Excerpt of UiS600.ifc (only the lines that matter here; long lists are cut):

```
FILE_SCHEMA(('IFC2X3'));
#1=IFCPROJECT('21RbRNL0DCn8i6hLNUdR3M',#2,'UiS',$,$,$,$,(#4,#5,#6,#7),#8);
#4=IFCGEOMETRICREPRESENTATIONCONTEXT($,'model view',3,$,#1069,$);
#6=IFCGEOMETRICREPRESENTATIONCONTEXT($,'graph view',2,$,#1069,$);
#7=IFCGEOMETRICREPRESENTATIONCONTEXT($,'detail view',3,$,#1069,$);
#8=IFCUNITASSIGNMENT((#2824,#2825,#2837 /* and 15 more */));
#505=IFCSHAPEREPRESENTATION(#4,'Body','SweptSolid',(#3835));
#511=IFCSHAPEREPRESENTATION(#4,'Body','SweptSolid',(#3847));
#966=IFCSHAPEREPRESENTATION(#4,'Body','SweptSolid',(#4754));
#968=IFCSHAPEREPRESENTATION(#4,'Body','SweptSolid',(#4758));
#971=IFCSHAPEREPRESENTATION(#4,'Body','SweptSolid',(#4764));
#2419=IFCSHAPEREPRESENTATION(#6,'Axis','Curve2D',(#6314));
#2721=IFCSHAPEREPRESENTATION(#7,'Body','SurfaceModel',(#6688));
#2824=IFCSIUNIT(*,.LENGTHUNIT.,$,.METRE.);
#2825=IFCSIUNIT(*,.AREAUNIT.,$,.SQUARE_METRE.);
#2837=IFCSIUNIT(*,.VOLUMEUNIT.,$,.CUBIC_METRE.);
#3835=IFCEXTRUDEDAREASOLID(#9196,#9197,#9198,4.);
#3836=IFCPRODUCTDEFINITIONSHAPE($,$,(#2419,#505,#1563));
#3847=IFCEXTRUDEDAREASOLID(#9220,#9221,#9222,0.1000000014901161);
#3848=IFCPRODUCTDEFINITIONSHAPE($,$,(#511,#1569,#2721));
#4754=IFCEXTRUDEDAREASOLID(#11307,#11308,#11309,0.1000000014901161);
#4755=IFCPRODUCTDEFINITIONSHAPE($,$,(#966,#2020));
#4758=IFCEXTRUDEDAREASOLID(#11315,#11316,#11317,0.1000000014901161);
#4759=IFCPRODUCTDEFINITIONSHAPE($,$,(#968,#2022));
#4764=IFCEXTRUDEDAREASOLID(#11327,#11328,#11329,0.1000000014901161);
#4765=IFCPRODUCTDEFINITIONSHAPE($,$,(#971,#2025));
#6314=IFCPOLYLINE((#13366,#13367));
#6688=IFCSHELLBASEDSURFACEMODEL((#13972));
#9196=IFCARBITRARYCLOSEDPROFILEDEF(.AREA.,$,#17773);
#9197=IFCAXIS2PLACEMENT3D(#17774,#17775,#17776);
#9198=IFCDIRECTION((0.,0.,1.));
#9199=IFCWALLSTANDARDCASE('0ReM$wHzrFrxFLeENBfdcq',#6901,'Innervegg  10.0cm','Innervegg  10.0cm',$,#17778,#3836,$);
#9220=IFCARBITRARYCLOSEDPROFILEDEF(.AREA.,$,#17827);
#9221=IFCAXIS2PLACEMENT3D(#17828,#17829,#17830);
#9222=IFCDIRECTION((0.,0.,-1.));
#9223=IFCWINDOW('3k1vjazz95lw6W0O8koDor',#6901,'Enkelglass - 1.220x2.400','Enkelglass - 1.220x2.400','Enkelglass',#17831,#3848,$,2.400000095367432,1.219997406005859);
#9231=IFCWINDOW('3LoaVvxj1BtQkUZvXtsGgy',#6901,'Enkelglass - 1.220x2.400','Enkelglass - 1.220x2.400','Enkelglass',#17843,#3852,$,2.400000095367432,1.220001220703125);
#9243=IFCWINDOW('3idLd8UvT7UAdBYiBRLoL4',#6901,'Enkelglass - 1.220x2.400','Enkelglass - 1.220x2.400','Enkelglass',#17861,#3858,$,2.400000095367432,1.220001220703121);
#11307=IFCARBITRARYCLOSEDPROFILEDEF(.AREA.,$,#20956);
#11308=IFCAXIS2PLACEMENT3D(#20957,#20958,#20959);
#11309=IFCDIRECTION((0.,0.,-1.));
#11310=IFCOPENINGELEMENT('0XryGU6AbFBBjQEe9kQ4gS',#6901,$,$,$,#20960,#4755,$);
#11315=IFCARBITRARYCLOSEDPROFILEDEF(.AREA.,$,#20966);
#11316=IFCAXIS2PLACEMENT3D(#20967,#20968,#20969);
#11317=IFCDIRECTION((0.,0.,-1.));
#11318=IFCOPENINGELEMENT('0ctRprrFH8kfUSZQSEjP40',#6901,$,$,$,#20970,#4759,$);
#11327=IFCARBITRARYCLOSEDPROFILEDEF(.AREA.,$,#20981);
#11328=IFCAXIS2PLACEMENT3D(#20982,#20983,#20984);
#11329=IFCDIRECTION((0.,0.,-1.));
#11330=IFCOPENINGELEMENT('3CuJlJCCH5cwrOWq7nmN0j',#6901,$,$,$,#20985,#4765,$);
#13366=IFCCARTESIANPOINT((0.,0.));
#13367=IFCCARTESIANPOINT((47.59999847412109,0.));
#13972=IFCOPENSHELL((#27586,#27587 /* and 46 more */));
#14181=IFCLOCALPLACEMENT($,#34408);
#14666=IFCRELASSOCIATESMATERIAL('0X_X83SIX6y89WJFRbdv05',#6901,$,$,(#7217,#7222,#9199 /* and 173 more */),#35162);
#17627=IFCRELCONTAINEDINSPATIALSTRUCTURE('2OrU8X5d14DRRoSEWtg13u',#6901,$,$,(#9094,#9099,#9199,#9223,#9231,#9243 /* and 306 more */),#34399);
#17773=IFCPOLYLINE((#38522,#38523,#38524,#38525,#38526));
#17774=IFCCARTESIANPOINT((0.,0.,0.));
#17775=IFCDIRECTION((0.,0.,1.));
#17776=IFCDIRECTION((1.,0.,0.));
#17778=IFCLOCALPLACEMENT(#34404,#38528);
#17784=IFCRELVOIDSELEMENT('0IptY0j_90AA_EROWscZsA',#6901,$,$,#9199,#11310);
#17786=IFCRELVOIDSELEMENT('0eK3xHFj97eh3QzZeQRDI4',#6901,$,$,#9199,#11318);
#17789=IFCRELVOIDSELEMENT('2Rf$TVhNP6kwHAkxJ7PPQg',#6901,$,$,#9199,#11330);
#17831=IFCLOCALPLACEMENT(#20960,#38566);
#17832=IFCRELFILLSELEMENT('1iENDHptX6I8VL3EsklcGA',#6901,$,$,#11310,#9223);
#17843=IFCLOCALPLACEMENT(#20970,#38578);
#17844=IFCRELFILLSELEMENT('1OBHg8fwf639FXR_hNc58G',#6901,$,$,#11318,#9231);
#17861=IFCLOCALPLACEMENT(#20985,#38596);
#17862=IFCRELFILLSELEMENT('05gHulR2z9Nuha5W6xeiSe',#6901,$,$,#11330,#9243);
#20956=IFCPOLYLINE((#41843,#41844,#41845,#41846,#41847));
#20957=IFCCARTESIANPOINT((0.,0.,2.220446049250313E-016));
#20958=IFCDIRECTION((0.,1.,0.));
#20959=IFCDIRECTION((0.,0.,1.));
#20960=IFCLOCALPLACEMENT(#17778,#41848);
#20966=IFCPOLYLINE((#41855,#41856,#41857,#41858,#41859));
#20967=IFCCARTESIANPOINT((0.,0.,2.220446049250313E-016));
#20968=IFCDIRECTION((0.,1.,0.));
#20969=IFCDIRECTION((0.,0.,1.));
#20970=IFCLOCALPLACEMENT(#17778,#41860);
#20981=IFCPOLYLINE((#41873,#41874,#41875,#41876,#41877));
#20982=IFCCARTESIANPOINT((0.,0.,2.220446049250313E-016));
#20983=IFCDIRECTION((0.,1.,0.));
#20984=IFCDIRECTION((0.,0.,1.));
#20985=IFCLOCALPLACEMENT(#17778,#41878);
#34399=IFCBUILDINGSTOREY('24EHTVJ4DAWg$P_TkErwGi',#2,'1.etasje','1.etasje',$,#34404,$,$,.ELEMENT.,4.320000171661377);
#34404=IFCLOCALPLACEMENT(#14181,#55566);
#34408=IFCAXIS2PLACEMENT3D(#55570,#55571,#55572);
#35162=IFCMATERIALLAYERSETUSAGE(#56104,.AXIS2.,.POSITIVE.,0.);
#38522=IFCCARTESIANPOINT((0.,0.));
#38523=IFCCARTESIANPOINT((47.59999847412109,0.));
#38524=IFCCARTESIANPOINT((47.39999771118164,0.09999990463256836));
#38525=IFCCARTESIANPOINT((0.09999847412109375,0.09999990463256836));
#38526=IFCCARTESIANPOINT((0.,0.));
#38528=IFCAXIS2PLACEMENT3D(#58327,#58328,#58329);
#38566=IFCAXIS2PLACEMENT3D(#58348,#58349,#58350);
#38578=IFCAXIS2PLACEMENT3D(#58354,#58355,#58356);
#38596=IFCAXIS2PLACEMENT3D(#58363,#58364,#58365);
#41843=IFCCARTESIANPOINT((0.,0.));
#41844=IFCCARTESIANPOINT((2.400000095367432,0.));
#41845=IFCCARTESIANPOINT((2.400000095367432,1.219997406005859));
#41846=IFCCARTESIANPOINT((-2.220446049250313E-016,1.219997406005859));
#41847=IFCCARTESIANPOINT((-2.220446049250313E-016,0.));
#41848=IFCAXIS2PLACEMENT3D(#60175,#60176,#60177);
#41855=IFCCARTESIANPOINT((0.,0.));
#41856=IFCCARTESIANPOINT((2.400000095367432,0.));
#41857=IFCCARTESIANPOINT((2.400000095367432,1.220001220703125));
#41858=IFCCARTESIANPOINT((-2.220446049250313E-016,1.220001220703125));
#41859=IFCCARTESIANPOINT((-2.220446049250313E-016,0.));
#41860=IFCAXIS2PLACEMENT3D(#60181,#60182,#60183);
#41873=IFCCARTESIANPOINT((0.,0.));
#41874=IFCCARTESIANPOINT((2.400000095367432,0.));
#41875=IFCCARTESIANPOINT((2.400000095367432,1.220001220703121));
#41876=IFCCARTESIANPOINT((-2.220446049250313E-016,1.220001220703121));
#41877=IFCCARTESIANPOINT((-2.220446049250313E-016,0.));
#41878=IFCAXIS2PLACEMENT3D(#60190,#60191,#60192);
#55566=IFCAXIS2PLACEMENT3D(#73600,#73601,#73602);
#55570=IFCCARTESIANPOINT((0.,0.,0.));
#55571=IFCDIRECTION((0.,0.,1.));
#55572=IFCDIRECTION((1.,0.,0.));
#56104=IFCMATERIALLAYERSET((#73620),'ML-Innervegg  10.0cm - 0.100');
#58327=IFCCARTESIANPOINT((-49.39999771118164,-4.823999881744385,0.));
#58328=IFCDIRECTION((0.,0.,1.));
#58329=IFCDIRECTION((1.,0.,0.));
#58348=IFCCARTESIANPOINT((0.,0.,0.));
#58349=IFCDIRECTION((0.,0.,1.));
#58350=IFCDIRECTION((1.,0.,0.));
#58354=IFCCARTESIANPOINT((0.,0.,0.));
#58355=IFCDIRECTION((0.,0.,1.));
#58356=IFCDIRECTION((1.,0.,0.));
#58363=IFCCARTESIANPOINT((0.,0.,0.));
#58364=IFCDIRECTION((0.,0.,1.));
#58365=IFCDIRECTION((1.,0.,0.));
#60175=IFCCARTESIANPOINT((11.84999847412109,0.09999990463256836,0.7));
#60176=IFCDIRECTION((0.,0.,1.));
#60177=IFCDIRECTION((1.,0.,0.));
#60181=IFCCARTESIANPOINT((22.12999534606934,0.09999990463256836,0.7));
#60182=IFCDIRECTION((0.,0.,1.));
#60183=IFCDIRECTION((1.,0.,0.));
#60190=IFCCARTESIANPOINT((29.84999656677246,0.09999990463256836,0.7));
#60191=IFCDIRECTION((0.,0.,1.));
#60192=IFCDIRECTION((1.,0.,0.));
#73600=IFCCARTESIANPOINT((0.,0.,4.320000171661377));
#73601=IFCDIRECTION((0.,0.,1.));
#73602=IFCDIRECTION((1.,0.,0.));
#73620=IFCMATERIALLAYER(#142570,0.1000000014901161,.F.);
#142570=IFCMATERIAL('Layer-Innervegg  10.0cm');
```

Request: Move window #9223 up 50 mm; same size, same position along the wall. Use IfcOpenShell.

```python
import numpy as np
import ifcopenshell
import ifcopenshell.api.geometry
import ifcopenshell.util.placement
import ifcopenshell.util.unit

model = ifcopenshell.open("UiS600.ifc")
unit_scale = ifcopenshell.util.unit.calculate_unit_scale(model)

window = model.by_id(9223)
opening = window.FillsVoids[0].RelatingOpeningElement
dz = 0.05

shift = np.array([0.0, 0.0, dz])
# The window is placed relative to its opening, so it follows when the opening moves.
matrix = ifcopenshell.util.placement.get_local_placement(opening.ObjectPlacement)
matrix[:3, 3] += shift
ifcopenshell.api.geometry.edit_object_placement(
    model, product=opening, matrix=matrix, is_si=False, should_transform_children=True
)

print(f"moved by {dz * unit_scale:+.3f} m")

model.write("UiS600-out.ifc")
```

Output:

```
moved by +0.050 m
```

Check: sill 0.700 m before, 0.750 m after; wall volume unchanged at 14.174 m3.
